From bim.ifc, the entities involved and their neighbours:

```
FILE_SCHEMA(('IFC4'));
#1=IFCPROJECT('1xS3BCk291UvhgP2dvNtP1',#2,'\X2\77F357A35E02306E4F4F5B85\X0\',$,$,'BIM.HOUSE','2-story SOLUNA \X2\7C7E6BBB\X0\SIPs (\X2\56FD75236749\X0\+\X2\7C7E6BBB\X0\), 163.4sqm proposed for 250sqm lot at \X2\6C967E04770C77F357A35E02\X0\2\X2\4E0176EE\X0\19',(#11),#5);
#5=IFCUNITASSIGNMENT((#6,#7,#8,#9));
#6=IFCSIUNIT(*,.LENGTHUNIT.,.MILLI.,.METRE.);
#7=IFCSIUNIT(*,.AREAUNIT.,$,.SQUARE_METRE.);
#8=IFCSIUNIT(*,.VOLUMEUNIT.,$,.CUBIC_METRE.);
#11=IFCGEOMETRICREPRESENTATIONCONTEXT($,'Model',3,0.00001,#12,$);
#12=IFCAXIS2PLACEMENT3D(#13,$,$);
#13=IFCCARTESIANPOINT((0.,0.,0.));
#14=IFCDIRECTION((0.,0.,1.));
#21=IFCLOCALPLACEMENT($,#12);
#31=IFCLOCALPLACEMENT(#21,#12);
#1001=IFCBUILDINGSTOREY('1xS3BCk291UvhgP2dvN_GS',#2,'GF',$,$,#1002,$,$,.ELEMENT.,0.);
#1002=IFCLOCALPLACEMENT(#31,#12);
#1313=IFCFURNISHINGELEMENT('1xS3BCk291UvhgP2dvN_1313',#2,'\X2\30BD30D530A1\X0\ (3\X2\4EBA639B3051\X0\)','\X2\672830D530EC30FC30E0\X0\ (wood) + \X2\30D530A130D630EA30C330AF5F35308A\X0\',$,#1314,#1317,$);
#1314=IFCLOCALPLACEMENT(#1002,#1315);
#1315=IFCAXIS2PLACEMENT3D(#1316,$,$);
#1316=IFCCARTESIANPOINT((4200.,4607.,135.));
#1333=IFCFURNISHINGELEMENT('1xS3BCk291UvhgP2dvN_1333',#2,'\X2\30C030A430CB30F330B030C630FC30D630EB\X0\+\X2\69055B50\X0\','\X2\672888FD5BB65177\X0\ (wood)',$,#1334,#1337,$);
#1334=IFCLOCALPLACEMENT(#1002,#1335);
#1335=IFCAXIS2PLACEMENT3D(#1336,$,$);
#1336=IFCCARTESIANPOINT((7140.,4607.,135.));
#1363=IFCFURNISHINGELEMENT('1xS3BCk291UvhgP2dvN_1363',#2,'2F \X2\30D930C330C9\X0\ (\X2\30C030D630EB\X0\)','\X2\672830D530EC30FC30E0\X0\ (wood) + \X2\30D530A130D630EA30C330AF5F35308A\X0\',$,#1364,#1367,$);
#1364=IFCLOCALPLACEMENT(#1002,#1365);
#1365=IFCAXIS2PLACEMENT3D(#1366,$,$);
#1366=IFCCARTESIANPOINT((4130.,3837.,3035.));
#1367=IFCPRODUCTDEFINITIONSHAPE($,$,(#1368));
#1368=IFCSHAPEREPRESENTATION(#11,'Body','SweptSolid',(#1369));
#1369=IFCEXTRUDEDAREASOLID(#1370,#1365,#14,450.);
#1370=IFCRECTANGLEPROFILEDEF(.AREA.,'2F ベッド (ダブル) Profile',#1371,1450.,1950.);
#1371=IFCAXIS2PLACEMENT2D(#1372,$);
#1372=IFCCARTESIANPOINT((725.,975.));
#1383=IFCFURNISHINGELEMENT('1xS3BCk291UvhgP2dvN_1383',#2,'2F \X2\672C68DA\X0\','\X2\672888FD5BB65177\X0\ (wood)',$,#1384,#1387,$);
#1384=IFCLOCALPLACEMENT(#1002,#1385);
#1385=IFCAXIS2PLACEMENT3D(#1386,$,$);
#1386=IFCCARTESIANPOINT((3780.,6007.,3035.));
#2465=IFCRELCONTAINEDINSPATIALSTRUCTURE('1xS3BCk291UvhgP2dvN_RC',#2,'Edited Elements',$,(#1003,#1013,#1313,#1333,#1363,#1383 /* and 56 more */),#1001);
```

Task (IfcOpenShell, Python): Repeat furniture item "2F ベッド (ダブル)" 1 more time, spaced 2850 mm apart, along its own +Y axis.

```python
import ifcopenshell
import ifcopenshell.api.geometry
import ifcopenshell.api.root
import ifcopenshell.util.element
import ifcopenshell.util.placement
import ifcopenshell.util.unit

model = ifcopenshell.open("bim.ifc")
unit_scale = ifcopenshell.util.unit.calculate_unit_scale(model)


def reuse_history(source, copy):
    """copy_class also copies each property set's owner history, people and application; keep the originals."""
    for rel in copy.IsDefinedBy:
        if rel.is_a("IfcRelDefinesByProperties") and (history := rel.RelatingPropertyDefinition.OwnerHistory):
            rel.RelatingPropertyDefinition.OwnerHistory = source.OwnerHistory
            ifcopenshell.util.element.remove_deep2(model, history)


source = model.by_id(1363)
base = ifcopenshell.util.placement.get_local_placement(source.ObjectPlacement)
step = base[:3, 1] * 2.85 / unit_scale

for i in range(1, 2):
    copy = ifcopenshell.api.root.copy_class(model, product=source)
    copy.Representation = ifcopenshell.util.element.copy_deep(
        model, source.Representation, exclude=["IfcGeometricRepresentationContext", "IfcRepresentationMap"]
    )
    reuse_history(source, copy)
    matrix = base.copy()
    matrix[:3, 3] += i * step
    print("added at", matrix[:3, 3].round(3) + 0.0)
    ifcopenshell.api.geometry.edit_object_placement(model, product=copy, matrix=matrix, is_si=False)

model.write("bim_edited.ifc")
```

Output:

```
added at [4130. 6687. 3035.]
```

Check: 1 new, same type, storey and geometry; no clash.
